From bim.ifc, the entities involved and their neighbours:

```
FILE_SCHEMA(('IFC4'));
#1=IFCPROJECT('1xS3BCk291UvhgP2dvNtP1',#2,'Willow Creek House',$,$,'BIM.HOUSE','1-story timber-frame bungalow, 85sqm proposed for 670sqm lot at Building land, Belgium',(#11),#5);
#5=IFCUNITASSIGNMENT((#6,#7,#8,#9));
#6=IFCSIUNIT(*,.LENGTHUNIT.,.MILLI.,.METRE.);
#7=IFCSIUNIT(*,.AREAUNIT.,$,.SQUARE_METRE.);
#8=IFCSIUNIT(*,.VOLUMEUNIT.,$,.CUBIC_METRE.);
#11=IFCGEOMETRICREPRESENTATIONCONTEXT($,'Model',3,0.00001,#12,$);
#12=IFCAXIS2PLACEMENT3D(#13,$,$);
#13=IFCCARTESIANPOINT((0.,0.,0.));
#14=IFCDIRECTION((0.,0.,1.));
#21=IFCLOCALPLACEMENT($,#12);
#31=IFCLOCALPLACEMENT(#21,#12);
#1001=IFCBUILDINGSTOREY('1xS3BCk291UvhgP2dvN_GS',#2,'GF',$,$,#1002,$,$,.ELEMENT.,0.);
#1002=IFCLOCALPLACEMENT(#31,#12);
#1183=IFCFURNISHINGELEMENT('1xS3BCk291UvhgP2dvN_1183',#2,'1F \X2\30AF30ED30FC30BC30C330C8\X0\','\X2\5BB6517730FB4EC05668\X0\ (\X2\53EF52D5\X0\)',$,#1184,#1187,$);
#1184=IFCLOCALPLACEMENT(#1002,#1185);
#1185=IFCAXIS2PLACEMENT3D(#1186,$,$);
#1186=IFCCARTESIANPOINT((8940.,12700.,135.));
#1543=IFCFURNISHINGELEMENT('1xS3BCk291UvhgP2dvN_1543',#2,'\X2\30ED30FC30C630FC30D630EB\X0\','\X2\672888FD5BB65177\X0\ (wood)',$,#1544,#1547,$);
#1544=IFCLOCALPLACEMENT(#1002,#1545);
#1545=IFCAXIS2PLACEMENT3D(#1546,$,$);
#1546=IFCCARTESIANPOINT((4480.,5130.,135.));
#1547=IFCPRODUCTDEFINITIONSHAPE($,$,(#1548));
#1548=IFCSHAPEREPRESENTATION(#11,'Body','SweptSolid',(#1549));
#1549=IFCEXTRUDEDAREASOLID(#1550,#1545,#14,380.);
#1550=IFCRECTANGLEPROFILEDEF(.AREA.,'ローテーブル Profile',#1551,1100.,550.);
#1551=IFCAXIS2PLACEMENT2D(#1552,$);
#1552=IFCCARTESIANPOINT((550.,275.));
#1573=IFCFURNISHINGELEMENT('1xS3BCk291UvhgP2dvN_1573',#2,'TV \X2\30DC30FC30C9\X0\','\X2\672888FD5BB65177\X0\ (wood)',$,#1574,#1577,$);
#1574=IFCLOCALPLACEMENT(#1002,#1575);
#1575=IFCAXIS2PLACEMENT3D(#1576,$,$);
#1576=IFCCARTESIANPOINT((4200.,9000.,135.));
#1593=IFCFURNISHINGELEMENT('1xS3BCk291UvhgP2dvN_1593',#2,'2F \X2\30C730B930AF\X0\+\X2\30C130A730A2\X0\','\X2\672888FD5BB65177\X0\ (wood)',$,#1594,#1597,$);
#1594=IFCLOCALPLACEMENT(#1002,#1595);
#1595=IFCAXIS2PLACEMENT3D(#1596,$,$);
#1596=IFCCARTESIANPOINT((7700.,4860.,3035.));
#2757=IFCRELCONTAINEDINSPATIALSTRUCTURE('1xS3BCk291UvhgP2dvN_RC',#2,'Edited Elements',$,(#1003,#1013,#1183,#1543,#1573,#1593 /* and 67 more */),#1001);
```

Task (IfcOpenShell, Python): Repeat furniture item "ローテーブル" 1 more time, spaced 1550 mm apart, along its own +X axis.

```python
import ifcopenshell
import ifcopenshell.api.geometry
import ifcopenshell.api.root
import ifcopenshell.util.element
import ifcopenshell.util.placement

model = ifcopenshell.open("bim.ifc")


def reuse_history(source, copy):
    """copy_class also copies each property set's owner history, people and application; keep the originals."""
    for rel in copy.IsDefinedBy:
        if rel.is_a("IfcRelDefinesByProperties") and (history := rel.RelatingPropertyDefinition.OwnerHistory):
            rel.RelatingPropertyDefinition.OwnerHistory = source.OwnerHistory
            ifcopenshell.util.element.remove_deep2(model, history)


source = model.by_guid("1xS3BCk291UvhgP2dvN_1543")
base = ifcopenshell.util.placement.get_local_placement(source.ObjectPlacement)
step = base[:3, 0] * 1550.0

for i in range(1, 2):
    copy = ifcopenshell.api.root.copy_class(model, product=source)
    copy.Representation = ifcopenshell.util.element.copy_deep(
        model, source.Representation, exclude=["IfcGeometricRepresentationContext", "IfcRepresentationMap"]
    )
    reuse_history(source, copy)
    matrix = base.copy()
    matrix[:3, 3] += i * step
    print("added at", matrix[:3, 3].round(3) + 0.0)
    ifcopenshell.api.geometry.edit_object_placement(model, product=copy, matrix=matrix, is_si=False)

model.write("bim_updated.ifc")
```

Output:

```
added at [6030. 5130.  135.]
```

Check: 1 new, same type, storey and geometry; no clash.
